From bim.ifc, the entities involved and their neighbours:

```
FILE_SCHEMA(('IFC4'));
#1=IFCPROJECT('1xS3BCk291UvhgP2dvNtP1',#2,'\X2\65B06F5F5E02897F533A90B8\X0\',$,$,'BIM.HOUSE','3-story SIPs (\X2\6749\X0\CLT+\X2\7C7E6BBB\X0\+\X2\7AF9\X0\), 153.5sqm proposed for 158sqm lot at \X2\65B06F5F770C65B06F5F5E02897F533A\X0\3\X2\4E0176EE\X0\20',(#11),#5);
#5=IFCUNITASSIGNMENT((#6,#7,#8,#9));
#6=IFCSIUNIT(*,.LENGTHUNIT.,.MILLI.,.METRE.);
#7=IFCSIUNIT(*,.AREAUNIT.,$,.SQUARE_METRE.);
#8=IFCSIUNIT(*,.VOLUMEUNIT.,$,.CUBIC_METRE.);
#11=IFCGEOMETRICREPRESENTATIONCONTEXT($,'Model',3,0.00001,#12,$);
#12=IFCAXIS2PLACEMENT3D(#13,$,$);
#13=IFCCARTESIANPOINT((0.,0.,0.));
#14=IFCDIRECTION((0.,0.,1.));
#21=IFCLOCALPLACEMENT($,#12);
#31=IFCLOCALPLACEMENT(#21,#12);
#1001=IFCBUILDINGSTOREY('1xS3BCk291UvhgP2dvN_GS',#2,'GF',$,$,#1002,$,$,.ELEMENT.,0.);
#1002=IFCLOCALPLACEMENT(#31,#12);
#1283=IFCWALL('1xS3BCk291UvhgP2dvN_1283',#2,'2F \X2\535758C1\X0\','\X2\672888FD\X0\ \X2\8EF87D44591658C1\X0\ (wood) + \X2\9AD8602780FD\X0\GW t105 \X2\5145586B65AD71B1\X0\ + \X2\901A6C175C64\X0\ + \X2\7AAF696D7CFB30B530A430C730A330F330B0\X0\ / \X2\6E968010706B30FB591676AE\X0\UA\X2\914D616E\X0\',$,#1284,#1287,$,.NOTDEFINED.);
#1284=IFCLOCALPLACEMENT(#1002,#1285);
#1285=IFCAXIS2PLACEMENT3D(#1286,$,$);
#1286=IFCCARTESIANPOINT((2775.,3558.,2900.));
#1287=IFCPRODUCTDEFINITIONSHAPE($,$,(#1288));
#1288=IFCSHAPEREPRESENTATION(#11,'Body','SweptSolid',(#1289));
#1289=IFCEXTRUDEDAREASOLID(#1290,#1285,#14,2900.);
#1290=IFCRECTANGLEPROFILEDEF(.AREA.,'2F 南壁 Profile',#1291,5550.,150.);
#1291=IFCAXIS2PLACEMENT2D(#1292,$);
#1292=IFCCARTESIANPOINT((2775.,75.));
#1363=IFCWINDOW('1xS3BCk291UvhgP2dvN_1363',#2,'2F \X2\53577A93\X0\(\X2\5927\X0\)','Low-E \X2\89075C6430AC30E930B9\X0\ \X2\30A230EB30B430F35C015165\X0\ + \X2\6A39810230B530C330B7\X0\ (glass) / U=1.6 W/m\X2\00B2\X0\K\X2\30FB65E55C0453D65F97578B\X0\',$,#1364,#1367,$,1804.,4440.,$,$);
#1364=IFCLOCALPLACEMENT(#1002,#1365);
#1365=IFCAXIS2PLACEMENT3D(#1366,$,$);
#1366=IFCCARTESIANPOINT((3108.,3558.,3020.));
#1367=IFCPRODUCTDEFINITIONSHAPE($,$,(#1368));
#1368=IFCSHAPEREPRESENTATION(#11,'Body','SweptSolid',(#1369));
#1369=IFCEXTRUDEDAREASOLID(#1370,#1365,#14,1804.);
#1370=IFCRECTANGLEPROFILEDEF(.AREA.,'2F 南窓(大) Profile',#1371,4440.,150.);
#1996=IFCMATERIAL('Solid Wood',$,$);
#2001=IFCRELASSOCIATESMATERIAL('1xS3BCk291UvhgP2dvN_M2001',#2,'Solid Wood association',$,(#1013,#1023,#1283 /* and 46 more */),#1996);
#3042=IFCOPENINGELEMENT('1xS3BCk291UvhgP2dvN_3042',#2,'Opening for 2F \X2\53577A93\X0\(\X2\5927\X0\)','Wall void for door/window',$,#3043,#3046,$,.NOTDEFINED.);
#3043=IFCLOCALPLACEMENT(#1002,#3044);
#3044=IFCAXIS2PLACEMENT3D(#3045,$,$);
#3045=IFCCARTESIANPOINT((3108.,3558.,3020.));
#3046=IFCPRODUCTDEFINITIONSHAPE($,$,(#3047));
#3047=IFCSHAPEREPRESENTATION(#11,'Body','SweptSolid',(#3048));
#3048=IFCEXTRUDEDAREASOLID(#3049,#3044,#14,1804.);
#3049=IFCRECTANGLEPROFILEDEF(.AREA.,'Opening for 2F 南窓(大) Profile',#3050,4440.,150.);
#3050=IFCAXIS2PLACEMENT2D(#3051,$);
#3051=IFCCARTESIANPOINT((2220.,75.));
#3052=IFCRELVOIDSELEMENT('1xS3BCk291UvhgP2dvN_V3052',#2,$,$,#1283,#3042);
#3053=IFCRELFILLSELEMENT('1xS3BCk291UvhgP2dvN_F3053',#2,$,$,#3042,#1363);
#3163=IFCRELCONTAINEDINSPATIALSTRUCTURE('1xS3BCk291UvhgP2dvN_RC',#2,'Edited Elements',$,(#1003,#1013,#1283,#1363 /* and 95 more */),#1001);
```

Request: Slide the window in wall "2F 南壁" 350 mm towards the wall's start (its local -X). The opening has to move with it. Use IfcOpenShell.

```python
import ifcopenshell
import ifcopenshell.api.geometry
import ifcopenshell.util.placement
import ifcopenshell.util.unit

model = ifcopenshell.open("bim.ifc")
unit_scale = ifcopenshell.util.unit.calculate_unit_scale(model)

window = model.by_id(1363)
opening = window.FillsVoids[0].RelatingOpeningElement
wall = opening.VoidsElements[0].RelatingBuildingElement

wall_matrix = ifcopenshell.util.placement.get_local_placement(wall.ObjectPlacement)
shift = wall_matrix[:3, 0] * -0.35 / unit_scale
before = ifcopenshell.util.placement.get_local_placement(window.ObjectPlacement)[:3, 3].copy()

# The window is not placed relative to its opening, so move both.
for product in (opening, window):
    matrix = ifcopenshell.util.placement.get_local_placement(product.ObjectPlacement)
    matrix[:3, 3] += shift
    ifcopenshell.api.geometry.edit_object_placement(model, product=product, matrix=matrix, is_si=False)

after = ifcopenshell.util.placement.get_local_placement(window.ObjectPlacement)[:3, 3]
print("window moved by", (after - before).round(3) + 0.0)

model.write("bim_rev.ifc")
```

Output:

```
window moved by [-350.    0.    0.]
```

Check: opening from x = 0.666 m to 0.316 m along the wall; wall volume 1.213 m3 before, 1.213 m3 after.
